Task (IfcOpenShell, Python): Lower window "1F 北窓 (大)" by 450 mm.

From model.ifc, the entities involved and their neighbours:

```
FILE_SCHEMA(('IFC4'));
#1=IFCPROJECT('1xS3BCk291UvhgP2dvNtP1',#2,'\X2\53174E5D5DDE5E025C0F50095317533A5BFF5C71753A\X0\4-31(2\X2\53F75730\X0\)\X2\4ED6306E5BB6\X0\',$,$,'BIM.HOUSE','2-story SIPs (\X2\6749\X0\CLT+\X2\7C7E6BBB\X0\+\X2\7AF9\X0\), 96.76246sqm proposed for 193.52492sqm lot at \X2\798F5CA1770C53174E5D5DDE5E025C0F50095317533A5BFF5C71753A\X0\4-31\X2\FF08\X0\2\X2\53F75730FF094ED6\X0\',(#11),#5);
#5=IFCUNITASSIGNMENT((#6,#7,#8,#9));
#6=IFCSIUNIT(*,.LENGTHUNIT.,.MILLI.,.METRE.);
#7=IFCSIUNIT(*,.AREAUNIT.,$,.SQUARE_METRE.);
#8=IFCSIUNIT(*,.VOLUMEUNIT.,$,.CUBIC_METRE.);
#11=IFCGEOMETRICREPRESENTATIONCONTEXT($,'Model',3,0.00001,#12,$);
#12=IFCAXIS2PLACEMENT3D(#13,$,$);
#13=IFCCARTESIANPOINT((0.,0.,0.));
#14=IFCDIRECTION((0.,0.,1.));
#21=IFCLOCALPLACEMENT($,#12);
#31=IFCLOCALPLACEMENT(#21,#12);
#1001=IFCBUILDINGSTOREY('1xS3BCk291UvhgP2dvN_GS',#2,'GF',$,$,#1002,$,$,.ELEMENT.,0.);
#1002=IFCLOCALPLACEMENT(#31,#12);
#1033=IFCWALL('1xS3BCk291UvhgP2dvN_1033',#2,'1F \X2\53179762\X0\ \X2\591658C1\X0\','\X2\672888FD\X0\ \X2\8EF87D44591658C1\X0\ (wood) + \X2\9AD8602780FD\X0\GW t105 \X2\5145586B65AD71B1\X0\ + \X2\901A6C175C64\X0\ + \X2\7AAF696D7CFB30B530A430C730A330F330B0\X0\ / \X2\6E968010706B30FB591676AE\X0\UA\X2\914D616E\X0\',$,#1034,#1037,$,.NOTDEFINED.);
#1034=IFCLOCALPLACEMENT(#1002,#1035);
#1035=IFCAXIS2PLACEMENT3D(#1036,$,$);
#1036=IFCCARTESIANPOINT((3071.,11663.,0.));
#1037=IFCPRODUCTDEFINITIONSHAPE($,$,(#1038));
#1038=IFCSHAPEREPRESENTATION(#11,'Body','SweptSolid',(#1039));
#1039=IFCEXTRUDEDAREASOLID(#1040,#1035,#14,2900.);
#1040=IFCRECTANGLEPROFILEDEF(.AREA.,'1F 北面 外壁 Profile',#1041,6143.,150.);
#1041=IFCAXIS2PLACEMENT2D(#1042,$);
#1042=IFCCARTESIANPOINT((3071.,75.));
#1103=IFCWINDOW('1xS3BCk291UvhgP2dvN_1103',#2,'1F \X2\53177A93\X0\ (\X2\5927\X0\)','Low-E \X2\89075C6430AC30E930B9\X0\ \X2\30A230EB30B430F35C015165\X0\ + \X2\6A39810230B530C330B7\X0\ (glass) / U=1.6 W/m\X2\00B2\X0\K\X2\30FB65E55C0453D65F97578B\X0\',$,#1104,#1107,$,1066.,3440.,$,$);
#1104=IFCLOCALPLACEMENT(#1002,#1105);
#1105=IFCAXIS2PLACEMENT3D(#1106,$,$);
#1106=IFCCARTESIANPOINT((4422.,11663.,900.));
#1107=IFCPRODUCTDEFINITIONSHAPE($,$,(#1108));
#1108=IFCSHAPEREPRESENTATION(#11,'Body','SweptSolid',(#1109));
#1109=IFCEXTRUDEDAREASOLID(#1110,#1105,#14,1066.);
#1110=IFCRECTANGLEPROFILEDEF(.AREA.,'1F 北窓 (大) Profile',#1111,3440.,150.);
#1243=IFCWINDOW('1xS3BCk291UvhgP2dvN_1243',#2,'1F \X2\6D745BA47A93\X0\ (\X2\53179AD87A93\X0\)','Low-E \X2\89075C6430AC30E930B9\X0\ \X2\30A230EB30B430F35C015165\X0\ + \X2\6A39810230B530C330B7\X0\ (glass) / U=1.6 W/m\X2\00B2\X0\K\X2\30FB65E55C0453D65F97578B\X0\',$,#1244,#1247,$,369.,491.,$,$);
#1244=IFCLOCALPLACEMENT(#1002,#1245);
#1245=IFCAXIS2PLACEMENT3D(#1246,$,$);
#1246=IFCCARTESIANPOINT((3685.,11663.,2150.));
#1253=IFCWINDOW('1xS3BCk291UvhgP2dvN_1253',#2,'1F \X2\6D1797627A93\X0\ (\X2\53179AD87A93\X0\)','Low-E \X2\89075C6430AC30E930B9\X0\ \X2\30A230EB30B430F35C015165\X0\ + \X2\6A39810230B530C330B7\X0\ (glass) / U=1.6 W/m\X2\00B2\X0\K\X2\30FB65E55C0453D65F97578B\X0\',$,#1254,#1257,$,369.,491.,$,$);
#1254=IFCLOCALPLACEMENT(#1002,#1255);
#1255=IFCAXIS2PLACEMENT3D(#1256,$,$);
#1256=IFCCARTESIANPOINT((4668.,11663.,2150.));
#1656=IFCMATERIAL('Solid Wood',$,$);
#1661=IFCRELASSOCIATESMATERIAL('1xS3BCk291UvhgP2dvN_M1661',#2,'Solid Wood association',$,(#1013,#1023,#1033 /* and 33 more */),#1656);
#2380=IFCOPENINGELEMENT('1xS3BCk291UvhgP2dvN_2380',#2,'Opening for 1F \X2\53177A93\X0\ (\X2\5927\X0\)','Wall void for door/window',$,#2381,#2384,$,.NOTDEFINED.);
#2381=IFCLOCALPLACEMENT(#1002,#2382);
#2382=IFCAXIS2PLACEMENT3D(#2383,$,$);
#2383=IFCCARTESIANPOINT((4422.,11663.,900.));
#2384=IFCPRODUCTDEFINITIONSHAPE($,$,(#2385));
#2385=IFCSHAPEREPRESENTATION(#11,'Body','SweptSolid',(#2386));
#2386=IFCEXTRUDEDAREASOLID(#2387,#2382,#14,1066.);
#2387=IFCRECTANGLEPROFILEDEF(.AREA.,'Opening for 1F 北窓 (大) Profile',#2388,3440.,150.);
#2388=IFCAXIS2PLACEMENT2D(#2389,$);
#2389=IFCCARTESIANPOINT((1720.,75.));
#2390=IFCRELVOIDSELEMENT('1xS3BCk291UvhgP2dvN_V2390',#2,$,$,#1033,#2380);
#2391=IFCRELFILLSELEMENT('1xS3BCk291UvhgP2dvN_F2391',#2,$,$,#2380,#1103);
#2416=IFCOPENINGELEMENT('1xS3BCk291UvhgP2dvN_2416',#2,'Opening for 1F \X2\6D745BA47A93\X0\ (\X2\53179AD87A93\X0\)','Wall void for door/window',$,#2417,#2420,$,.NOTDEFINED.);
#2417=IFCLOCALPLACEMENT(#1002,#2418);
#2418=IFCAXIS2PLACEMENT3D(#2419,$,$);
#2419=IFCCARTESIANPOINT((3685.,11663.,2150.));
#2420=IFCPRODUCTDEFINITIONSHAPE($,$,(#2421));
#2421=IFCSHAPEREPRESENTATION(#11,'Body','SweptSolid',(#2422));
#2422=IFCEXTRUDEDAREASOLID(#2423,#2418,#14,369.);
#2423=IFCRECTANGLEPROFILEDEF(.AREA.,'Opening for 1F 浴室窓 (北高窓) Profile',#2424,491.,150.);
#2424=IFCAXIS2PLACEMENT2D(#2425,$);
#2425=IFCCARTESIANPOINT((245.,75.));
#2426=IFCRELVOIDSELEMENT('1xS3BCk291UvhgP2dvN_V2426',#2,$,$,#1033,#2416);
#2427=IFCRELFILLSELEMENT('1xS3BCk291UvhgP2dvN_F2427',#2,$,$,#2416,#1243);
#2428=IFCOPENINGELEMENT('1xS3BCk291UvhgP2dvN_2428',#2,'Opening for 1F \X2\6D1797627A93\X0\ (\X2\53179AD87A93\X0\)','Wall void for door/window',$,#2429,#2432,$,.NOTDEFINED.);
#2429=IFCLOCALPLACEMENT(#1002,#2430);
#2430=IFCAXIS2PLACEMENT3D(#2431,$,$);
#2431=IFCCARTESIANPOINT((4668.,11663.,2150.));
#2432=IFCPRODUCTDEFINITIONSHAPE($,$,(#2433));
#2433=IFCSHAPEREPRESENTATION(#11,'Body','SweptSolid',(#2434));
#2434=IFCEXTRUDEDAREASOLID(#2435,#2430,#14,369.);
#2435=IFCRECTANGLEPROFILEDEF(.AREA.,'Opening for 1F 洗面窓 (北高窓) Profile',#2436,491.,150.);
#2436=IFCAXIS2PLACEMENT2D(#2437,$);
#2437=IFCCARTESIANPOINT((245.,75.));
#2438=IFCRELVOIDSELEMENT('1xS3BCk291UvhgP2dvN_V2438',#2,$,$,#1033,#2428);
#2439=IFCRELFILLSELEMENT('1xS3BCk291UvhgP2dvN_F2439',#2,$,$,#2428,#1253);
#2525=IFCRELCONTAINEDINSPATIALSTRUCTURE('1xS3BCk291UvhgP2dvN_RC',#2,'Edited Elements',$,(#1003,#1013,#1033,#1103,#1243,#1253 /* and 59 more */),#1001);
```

```python
import numpy as np
import ifcopenshell
import ifcopenshell.api.geometry
import ifcopenshell.util.placement
import ifcopenshell.util.unit

model = ifcopenshell.open("model.ifc")
unit_scale = ifcopenshell.util.unit.calculate_unit_scale(model)

window = model.by_guid("1xS3BCk291UvhgP2dvN_1103")
opening = window.FillsVoids[0].RelatingOpeningElement
dz = -0.45 / unit_scale

shift = np.array([0.0, 0.0, dz])
# The window is not placed relative to its opening, so move both.
for product in (opening, window):
    matrix = ifcopenshell.util.placement.get_local_placement(product.ObjectPlacement)
    matrix[:3, 3] += shift
    ifcopenshell.api.geometry.edit_object_placement(model, product=product, matrix=matrix, is_si=False)

print(f"moved by {dz * unit_scale:+.3f} m")

model.write("model_updated.ifc")
```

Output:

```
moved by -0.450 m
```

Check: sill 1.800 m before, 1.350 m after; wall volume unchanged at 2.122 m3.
